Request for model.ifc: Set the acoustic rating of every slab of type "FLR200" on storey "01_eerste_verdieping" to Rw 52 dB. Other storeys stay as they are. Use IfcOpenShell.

First a look at what the model holds.

```python
import ifcopenshell
import ifcopenshell.util.element

model = ifcopenshell.open("model.ifc")
print(model.schema)
storey = next(s for s in model.by_type("IfcBuildingStorey") if s.Name == "01_eerste_verdieping")
slabs = [e for e in ifcopenshell.util.element.get_decomposition(storey) if e.is_a("IfcSlab")]
seen = {}
for e in slabs:
    element_type = ifcopenshell.util.element.get_type(e)
    key = (element_type.Name if element_type != e and element_type else None, ifcopenshell.util.element.get_pset(e, "Pset_SlabCommon", "AcousticRating"))
    seen[key] = seen.get(key, 0) + 1
for (name, value), count in sorted(seen.items(), key=str):
    print(count, "x", name, "|", value)
```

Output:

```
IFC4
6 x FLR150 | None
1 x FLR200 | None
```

```python
import ifcopenshell
import ifcopenshell.api.pset
import ifcopenshell.util.element

model = ifcopenshell.open("model.ifc")

storey = next(s for s in model.by_type("IfcBuildingStorey") if s.Name == "01_eerste_verdieping")
slabs = [e for e in ifcopenshell.util.element.get_decomposition(storey) if e.is_a("IfcSlab")]

count = 0
for e in slabs:
    element_type = ifcopenshell.util.element.get_type(e)
    if element_type in (None, e) or element_type.Name != "FLR200":
        continue
    # add_pset returns the element's existing set when there is one.
    pset = ifcopenshell.api.pset.add_pset(model, product=e, name="Pset_SlabCommon")
    ifcopenshell.api.pset.edit_pset(model, pset=pset, properties={"AcousticRating": "Rw 52 dB"})
    count += 1

print(count, "slabs updated")

model.write("model_updated.ifc")
```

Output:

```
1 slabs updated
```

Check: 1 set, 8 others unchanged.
